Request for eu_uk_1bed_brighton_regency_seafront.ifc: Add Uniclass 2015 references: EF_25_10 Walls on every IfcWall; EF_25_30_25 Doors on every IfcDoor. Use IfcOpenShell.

First a look at what the model holds.

```python
import ifcopenshell

model = ifcopenshell.open("eu_uk_1bed_brighton_regency_seafront.ifc")
print(model.schema)
print("classifications:", [c.Name for c in model.by_type("IfcClassification")])
for ifc_class in ("IfcDoor", "IfcRoof", "IfcStair", "IfcWall", "IfcWindow"):
    print(ifc_class, len(model.by_type(ifc_class)))
```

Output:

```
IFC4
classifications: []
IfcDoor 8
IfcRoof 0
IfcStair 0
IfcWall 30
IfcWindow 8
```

```python
import ifcopenshell
import ifcopenshell.api.classification

model = ifcopenshell.open("eu_uk_1bed_brighton_regency_seafront.ifc")

system = ifcopenshell.api.classification.add_classification(model, classification="Uniclass 2015")

codes = {
    "IfcWall": ("EF_25_10", "Walls"),
    "IfcDoor": ("EF_25_30_25", "Doors"),
}
for ifc_class, (code, name) in codes.items():
    products = model.by_type(ifc_class)
    ifcopenshell.api.classification.add_reference(
        model, products=products, classification=system, identification=code, name=name
    )
    print(code, len(products))

model.write("eu_uk_1bed_brighton_regency_seafront_v2.ifc")
```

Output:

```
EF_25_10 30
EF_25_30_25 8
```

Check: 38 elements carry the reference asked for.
